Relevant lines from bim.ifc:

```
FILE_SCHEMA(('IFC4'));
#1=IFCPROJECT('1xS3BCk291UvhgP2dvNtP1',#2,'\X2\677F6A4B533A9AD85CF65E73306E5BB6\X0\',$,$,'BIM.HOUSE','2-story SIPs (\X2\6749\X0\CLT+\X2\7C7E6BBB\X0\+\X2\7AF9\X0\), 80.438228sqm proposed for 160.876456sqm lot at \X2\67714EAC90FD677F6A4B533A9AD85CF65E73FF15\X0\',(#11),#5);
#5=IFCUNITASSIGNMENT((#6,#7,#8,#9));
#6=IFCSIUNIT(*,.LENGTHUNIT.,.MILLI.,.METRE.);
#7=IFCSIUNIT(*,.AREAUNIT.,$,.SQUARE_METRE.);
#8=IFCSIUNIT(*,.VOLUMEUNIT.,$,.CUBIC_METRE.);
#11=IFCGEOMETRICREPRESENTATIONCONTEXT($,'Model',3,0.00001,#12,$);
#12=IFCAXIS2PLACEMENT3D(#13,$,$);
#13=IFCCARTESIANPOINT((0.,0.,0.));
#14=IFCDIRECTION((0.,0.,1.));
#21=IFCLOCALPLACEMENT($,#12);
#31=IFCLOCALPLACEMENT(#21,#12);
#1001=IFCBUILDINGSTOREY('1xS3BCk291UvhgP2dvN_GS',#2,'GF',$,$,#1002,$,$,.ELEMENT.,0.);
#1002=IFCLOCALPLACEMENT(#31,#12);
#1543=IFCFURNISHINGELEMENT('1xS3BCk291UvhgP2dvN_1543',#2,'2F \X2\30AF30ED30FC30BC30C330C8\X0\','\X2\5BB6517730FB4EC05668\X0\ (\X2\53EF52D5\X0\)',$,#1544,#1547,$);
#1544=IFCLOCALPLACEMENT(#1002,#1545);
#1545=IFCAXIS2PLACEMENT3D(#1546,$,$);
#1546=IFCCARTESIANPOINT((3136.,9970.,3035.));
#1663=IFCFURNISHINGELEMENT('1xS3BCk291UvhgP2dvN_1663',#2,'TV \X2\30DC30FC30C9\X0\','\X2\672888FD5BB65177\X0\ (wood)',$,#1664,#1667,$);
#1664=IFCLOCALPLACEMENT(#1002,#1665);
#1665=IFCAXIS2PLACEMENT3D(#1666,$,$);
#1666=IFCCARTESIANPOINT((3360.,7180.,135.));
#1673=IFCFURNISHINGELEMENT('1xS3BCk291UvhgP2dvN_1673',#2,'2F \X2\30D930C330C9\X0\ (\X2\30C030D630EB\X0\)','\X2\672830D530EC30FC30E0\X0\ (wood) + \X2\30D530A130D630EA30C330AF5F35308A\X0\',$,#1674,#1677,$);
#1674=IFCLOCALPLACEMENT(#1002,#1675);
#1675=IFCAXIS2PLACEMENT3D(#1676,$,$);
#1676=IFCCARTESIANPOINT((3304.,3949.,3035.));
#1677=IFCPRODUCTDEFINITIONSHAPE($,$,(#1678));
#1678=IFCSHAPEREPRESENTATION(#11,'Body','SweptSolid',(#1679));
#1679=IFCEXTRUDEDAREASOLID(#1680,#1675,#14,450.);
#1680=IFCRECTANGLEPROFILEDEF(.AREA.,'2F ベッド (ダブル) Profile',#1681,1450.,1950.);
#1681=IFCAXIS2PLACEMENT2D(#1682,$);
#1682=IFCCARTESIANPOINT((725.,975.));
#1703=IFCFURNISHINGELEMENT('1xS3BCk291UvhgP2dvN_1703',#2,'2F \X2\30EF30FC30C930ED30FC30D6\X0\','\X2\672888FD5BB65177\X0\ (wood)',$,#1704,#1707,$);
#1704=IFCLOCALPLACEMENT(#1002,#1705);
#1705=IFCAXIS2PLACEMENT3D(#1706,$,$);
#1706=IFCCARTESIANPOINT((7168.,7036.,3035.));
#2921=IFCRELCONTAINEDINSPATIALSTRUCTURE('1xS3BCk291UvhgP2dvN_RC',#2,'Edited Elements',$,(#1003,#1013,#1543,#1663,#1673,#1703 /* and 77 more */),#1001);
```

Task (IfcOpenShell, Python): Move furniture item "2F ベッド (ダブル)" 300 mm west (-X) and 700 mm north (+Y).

```python
import ifcopenshell
import ifcopenshell.api.geometry
import ifcopenshell.util.placement
import ifcopenshell.util.unit

model = ifcopenshell.open("bim.ifc")
unit_scale = ifcopenshell.util.unit.calculate_unit_scale(model)

item = model.by_id(1673)
matrix = ifcopenshell.util.placement.get_local_placement(item.ObjectPlacement)
matrix[0, 3] -= 0.3 / unit_scale
matrix[1, 3] += 0.7 / unit_scale
ifcopenshell.api.geometry.edit_object_placement(model, product=item, matrix=matrix, is_si=False)

print(ifcopenshell.util.placement.get_local_placement(item.ObjectPlacement).round(3) + 0.0)

model.write("bim_rev.ifc")
```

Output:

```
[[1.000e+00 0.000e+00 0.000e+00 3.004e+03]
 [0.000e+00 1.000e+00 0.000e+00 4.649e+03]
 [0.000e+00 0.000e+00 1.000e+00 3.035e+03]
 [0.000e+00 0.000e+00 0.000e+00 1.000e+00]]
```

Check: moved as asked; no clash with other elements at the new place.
